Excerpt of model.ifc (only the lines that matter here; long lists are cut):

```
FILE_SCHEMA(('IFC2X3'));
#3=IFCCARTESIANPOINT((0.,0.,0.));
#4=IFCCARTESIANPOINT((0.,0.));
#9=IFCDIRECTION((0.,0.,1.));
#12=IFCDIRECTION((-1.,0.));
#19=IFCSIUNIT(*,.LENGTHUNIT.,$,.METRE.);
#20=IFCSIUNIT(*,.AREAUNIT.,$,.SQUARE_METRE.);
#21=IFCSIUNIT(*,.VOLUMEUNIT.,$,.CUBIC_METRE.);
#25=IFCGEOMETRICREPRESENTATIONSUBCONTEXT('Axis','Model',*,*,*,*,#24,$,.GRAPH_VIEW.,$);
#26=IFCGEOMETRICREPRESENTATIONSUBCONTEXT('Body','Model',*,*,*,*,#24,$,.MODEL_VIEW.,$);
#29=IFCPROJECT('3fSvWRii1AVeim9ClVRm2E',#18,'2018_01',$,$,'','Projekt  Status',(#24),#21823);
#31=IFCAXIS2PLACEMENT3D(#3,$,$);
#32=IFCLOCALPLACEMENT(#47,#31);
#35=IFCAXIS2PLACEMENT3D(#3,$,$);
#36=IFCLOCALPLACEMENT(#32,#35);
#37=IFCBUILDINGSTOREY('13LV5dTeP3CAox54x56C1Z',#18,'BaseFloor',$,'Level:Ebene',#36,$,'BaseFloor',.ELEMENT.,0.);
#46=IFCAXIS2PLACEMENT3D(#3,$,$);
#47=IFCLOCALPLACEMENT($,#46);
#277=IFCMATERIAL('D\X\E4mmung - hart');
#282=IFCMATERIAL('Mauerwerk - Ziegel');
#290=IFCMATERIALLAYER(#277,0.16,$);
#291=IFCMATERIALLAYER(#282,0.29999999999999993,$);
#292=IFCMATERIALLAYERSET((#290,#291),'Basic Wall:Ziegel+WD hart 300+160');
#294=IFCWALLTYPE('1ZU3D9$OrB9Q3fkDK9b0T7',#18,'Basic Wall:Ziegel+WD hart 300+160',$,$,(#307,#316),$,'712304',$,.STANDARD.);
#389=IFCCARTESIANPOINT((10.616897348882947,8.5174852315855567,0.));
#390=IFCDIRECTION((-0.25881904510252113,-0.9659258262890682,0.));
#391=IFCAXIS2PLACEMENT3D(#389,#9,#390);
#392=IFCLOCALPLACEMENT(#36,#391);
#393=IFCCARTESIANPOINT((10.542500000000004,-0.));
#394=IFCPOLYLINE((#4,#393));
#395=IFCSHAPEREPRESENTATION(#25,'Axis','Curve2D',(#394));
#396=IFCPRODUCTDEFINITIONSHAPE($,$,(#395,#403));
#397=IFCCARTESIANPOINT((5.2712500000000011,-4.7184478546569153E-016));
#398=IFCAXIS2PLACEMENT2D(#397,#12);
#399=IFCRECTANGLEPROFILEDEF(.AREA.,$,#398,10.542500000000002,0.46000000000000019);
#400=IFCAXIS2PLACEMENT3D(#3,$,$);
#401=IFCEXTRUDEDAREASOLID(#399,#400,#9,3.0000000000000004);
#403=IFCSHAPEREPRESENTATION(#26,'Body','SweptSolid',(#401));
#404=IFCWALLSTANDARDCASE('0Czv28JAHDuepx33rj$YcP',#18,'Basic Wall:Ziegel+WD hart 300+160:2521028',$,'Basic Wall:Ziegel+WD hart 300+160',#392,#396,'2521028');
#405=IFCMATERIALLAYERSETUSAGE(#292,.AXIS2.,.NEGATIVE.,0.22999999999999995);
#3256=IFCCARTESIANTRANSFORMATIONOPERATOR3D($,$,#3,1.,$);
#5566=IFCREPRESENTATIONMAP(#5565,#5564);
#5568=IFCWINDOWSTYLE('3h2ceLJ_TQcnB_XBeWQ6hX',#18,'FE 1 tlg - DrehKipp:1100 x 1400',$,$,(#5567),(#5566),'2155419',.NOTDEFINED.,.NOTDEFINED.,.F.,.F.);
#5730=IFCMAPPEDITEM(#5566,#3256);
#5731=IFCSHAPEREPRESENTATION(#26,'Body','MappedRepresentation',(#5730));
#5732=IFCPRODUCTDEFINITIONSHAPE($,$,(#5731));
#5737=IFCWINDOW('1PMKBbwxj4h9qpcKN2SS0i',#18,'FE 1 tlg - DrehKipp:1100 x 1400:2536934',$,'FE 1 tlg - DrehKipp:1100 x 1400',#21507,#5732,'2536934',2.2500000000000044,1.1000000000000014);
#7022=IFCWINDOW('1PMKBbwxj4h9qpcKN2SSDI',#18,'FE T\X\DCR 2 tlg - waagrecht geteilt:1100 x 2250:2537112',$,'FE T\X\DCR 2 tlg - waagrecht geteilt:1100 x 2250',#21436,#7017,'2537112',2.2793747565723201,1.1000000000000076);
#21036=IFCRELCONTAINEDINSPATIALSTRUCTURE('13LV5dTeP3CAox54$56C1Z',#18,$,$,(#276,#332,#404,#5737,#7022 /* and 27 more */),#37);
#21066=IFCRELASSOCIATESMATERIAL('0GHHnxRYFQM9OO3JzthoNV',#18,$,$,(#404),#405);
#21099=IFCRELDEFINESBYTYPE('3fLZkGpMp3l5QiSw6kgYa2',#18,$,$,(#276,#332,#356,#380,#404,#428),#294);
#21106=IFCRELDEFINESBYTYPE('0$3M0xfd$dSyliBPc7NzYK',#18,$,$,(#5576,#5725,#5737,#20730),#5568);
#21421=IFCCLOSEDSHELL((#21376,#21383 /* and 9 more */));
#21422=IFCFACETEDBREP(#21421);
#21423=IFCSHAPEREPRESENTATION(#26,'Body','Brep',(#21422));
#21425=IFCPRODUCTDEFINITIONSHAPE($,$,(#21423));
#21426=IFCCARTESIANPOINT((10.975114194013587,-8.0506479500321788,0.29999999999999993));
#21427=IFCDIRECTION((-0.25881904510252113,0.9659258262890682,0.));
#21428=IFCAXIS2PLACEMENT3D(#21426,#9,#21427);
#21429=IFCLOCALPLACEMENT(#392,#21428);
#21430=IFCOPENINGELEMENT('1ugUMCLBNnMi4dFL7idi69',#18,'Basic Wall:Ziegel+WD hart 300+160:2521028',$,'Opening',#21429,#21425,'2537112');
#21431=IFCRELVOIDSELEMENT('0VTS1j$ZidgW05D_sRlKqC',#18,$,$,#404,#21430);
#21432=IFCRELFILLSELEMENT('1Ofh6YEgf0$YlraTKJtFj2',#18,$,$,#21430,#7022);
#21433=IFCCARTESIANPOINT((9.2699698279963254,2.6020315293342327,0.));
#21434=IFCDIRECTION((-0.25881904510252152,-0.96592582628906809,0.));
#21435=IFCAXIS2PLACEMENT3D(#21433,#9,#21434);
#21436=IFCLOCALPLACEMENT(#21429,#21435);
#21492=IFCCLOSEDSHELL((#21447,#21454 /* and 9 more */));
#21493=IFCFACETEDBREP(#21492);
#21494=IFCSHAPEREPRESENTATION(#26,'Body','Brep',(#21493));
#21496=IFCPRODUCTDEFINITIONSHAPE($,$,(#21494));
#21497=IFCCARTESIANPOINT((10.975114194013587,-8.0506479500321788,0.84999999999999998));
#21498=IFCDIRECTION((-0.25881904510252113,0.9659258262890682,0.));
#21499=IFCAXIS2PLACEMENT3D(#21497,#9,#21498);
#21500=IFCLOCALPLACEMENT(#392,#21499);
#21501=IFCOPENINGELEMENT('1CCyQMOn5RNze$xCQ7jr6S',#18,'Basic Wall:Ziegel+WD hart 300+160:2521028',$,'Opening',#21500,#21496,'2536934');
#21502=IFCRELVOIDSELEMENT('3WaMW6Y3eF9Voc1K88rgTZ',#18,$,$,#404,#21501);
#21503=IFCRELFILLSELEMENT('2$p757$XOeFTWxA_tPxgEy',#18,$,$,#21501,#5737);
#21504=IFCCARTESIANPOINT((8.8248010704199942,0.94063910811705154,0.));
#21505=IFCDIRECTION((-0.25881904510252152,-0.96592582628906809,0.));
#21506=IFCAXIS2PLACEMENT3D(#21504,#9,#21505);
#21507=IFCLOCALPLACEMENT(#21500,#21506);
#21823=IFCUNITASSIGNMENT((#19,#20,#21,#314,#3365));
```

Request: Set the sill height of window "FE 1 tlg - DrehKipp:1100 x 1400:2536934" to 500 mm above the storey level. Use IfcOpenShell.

```python
import numpy as np
import ifcopenshell
import ifcopenshell.api.geometry
import ifcopenshell.geom
import ifcopenshell.util.element
import ifcopenshell.util.placement
import ifcopenshell.util.shape
import ifcopenshell.util.unit

model = ifcopenshell.open("model.ifc")
unit_scale = ifcopenshell.util.unit.calculate_unit_scale(model)

window = model.by_guid("1PMKBbwxj4h9qpcKN2SS0i")
opening = window.FillsVoids[0].RelatingOpeningElement
storey = ifcopenshell.util.element.get_container(window, ifc_class="IfcBuildingStorey")
level = ifcopenshell.util.placement.get_local_placement(storey.ObjectPlacement)[2, 3]

# The opening's origin need not be at the sill, so measure its lowest point.
shape = ifcopenshell.geom.create_shape(ifcopenshell.geom.settings(), opening)
bottom = ifcopenshell.util.shape.get_shape_bottom_elevation(shape, shape.geometry) / unit_scale
dz = level + 0.5 - bottom

shift = np.array([0.0, 0.0, dz])
# The window is placed relative to its opening, so it follows when the opening moves.
matrix = ifcopenshell.util.placement.get_local_placement(opening.ObjectPlacement)
matrix[:3, 3] += shift
ifcopenshell.api.geometry.edit_object_placement(
    model, product=opening, matrix=matrix, is_si=False, should_transform_children=True
)

print(f"moved by {dz * unit_scale:+.3f} m")

model.write("model_updated.ifc")
```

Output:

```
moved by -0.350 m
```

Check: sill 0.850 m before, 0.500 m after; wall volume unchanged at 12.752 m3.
